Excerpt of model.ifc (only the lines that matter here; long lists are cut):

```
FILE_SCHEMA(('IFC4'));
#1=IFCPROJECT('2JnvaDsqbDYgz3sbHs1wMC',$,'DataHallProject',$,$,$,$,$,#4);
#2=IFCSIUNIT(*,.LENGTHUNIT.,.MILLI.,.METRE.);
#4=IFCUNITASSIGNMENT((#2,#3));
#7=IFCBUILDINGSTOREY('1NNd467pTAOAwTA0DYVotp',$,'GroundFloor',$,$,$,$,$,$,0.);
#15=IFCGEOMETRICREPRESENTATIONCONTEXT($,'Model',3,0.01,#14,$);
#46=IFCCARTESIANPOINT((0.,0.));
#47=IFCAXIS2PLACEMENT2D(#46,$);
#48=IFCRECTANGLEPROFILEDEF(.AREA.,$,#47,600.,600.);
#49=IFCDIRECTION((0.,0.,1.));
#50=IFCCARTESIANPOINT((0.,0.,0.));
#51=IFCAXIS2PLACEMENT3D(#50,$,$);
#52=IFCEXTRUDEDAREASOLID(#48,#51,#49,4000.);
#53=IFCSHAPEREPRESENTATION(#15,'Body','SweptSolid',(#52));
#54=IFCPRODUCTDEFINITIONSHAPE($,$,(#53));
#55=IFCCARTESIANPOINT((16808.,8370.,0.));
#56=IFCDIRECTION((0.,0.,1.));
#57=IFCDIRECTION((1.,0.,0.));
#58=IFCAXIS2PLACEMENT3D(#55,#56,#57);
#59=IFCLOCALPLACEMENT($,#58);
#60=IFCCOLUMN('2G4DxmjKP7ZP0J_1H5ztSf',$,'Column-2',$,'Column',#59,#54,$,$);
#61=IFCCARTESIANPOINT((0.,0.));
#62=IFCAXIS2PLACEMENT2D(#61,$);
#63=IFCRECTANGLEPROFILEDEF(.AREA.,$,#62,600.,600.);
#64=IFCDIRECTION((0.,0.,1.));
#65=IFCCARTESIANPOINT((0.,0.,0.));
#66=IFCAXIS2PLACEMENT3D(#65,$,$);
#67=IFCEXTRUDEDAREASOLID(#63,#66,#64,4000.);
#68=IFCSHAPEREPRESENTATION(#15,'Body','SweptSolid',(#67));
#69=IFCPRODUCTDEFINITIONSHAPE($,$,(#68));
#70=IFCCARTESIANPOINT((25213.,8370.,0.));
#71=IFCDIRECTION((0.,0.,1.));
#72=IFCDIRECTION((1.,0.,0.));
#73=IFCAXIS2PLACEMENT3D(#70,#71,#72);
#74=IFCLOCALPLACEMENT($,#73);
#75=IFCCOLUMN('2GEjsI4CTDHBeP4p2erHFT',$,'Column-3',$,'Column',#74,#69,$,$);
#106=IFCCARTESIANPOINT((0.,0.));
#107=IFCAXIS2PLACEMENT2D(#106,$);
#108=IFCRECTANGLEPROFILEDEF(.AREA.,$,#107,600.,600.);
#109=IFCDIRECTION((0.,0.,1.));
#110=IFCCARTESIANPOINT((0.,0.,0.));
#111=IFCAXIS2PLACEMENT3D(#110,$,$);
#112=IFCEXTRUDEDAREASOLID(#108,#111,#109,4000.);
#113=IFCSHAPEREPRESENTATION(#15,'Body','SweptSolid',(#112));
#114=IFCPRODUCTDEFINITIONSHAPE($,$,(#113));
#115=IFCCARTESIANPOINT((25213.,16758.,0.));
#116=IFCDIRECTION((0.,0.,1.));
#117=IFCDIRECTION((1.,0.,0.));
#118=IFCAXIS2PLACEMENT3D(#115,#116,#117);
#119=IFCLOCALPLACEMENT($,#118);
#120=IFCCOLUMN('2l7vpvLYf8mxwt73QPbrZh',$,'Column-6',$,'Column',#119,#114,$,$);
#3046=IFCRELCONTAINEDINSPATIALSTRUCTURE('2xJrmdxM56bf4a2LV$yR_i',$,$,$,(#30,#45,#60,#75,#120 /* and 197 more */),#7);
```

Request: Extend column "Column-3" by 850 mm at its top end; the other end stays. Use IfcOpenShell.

```python
import ifcopenshell

model = ifcopenshell.open("model.ifc")

member = model.by_id(75)
change = 850.0

# The extrusion runs towards the end named, so only its depth changes.
body = next(r for r in member.Representation.Representations if r.RepresentationIdentifier == "Body")
solid = body.Items[0]
old_length = solid.Depth
solid.Depth += change

print(f"length {old_length:g} -> {solid.Depth:g}")

model.write("model-out.ifc")
```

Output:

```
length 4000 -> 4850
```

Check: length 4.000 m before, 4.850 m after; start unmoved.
